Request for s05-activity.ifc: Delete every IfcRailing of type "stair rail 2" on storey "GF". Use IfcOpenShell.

First a look at what the model holds.

```python
import ifcopenshell
import ifcopenshell.util.element

model = ifcopenshell.open("s05-activity.ifc")
print(model.schema)
storey = next(s for s in model.by_type("IfcBuildingStorey") if s.Name == "GF")
railings = [e for e in ifcopenshell.util.element.get_decomposition(storey) if e.is_a("IfcRailing")]
seen = {}
for e in railings:
    element_type = ifcopenshell.util.element.get_type(e)
    name = element_type.Name if element_type not in (None, e) else None
    seen[name] = seen.get(name, 0) + 1
for name, count in sorted(seen.items(), key=str):
    print(count, "x", name)
```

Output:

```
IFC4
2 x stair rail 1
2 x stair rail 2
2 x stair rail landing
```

```python
import ifcopenshell
import ifcopenshell.api.root
import ifcopenshell.util.element

model = ifcopenshell.open("s05-activity.ifc")

storey = next(s for s in model.by_type("IfcBuildingStorey") if s.Name == "GF")
railings = [e for e in ifcopenshell.util.element.get_decomposition(storey) if e.is_a("IfcRailing")]
targets = [e for e in railings if (t := ifcopenshell.util.element.get_type(e)) not in (None, e) and t.Name == "stair rail 2"]

for e in targets:
    ifcopenshell.api.root.remove_product(model, product=e)
print(len(targets), "removed")

model.write("s05-activity_updated.ifc")
```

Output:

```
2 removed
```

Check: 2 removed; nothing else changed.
